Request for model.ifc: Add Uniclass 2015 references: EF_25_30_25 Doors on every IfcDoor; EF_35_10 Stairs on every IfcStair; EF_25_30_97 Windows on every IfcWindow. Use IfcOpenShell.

First a look at what the model holds.

```python
import ifcopenshell

model = ifcopenshell.open("model.ifc")
print(model.schema)
print("classifications:", [c.Name for c in model.by_type("IfcClassification")])
for ifc_class in ("IfcDoor", "IfcRoof", "IfcStair", "IfcWall", "IfcWindow"):
    print(ifc_class, len(model.by_type(ifc_class)))
```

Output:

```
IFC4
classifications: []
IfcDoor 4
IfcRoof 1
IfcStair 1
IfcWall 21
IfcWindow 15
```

```python
import ifcopenshell
import ifcopenshell.api.classification

model = ifcopenshell.open("model.ifc")

system = ifcopenshell.api.classification.add_classification(model, classification="Uniclass 2015")

codes = {
    "IfcDoor": ("EF_25_30_25", "Doors"),
    "IfcStair": ("EF_35_10", "Stairs"),
    "IfcWindow": ("EF_25_30_97", "Windows"),
}
for ifc_class, (code, name) in codes.items():
    products = model.by_type(ifc_class)
    ifcopenshell.api.classification.add_reference(
        model, products=products, classification=system, identification=code, name=name
    )
    print(code, len(products))

model.write("model_updated.ifc")
```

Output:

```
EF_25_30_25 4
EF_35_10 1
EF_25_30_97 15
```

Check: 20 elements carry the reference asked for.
